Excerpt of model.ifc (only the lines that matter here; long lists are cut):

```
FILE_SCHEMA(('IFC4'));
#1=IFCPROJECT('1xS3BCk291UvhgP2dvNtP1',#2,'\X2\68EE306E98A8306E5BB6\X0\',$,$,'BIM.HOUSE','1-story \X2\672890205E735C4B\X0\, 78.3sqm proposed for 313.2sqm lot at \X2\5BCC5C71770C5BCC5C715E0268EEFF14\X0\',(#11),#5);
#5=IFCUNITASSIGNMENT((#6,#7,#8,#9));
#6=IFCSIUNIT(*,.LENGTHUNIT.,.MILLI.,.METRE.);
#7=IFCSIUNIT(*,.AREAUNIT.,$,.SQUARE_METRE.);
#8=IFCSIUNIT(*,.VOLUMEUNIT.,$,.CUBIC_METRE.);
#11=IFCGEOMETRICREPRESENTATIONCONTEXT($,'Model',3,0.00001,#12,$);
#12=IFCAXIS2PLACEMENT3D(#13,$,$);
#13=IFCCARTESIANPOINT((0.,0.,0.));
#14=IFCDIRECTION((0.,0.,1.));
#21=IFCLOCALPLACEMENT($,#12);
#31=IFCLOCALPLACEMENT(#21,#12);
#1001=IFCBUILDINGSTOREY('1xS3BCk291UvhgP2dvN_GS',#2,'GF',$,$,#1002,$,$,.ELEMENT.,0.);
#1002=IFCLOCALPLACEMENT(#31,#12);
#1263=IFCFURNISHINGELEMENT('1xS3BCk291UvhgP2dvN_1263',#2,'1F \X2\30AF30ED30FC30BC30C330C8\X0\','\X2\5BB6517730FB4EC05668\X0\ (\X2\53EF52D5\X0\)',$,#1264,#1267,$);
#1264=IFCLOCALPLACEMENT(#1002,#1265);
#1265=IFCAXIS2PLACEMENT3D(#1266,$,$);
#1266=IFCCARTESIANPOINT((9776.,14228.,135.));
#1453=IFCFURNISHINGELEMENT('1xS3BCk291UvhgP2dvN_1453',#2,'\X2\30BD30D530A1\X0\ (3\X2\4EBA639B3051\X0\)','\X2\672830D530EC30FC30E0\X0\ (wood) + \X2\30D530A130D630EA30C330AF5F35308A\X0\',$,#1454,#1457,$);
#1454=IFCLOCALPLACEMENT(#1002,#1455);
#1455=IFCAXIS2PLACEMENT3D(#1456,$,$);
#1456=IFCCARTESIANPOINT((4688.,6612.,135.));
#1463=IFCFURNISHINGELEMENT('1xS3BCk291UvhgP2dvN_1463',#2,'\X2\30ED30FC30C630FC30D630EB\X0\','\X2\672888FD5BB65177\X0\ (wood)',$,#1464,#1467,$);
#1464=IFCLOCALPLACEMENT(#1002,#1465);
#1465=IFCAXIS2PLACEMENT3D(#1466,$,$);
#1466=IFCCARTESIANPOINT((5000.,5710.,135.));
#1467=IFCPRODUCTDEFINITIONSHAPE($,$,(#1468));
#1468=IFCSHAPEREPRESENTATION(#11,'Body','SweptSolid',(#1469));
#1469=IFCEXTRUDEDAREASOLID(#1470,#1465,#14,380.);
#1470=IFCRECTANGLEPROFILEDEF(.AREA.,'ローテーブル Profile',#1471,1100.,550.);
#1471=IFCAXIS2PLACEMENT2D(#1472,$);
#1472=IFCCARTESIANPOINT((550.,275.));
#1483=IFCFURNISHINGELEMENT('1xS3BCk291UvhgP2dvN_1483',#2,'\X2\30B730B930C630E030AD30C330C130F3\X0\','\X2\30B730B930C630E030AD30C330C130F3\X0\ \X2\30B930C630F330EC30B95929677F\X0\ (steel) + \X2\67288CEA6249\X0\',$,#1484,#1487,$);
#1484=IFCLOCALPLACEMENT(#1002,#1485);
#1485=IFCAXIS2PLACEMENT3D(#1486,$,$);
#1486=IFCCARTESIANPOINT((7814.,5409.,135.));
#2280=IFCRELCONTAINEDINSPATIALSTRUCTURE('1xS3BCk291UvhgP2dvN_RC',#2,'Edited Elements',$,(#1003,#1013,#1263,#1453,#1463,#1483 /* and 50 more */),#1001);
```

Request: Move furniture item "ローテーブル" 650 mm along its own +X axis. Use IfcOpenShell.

```python
import ifcopenshell
import ifcopenshell.api.geometry
import ifcopenshell.util.placement
import ifcopenshell.util.unit

model = ifcopenshell.open("model.ifc")
unit_scale = ifcopenshell.util.unit.calculate_unit_scale(model)

item = model.by_id(1463)
matrix = ifcopenshell.util.placement.get_local_placement(item.ObjectPlacement)
matrix[:3, 3] += matrix[:3, 0] * 0.65 / unit_scale
ifcopenshell.api.geometry.edit_object_placement(model, product=item, matrix=matrix, is_si=False)

print(ifcopenshell.util.placement.get_local_placement(item.ObjectPlacement).round(3) + 0.0)

model.write("model_edited.ifc")
```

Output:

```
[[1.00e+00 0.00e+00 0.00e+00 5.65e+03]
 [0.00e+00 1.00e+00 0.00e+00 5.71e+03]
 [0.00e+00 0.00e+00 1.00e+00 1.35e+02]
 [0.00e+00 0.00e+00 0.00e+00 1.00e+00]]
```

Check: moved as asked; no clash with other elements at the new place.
